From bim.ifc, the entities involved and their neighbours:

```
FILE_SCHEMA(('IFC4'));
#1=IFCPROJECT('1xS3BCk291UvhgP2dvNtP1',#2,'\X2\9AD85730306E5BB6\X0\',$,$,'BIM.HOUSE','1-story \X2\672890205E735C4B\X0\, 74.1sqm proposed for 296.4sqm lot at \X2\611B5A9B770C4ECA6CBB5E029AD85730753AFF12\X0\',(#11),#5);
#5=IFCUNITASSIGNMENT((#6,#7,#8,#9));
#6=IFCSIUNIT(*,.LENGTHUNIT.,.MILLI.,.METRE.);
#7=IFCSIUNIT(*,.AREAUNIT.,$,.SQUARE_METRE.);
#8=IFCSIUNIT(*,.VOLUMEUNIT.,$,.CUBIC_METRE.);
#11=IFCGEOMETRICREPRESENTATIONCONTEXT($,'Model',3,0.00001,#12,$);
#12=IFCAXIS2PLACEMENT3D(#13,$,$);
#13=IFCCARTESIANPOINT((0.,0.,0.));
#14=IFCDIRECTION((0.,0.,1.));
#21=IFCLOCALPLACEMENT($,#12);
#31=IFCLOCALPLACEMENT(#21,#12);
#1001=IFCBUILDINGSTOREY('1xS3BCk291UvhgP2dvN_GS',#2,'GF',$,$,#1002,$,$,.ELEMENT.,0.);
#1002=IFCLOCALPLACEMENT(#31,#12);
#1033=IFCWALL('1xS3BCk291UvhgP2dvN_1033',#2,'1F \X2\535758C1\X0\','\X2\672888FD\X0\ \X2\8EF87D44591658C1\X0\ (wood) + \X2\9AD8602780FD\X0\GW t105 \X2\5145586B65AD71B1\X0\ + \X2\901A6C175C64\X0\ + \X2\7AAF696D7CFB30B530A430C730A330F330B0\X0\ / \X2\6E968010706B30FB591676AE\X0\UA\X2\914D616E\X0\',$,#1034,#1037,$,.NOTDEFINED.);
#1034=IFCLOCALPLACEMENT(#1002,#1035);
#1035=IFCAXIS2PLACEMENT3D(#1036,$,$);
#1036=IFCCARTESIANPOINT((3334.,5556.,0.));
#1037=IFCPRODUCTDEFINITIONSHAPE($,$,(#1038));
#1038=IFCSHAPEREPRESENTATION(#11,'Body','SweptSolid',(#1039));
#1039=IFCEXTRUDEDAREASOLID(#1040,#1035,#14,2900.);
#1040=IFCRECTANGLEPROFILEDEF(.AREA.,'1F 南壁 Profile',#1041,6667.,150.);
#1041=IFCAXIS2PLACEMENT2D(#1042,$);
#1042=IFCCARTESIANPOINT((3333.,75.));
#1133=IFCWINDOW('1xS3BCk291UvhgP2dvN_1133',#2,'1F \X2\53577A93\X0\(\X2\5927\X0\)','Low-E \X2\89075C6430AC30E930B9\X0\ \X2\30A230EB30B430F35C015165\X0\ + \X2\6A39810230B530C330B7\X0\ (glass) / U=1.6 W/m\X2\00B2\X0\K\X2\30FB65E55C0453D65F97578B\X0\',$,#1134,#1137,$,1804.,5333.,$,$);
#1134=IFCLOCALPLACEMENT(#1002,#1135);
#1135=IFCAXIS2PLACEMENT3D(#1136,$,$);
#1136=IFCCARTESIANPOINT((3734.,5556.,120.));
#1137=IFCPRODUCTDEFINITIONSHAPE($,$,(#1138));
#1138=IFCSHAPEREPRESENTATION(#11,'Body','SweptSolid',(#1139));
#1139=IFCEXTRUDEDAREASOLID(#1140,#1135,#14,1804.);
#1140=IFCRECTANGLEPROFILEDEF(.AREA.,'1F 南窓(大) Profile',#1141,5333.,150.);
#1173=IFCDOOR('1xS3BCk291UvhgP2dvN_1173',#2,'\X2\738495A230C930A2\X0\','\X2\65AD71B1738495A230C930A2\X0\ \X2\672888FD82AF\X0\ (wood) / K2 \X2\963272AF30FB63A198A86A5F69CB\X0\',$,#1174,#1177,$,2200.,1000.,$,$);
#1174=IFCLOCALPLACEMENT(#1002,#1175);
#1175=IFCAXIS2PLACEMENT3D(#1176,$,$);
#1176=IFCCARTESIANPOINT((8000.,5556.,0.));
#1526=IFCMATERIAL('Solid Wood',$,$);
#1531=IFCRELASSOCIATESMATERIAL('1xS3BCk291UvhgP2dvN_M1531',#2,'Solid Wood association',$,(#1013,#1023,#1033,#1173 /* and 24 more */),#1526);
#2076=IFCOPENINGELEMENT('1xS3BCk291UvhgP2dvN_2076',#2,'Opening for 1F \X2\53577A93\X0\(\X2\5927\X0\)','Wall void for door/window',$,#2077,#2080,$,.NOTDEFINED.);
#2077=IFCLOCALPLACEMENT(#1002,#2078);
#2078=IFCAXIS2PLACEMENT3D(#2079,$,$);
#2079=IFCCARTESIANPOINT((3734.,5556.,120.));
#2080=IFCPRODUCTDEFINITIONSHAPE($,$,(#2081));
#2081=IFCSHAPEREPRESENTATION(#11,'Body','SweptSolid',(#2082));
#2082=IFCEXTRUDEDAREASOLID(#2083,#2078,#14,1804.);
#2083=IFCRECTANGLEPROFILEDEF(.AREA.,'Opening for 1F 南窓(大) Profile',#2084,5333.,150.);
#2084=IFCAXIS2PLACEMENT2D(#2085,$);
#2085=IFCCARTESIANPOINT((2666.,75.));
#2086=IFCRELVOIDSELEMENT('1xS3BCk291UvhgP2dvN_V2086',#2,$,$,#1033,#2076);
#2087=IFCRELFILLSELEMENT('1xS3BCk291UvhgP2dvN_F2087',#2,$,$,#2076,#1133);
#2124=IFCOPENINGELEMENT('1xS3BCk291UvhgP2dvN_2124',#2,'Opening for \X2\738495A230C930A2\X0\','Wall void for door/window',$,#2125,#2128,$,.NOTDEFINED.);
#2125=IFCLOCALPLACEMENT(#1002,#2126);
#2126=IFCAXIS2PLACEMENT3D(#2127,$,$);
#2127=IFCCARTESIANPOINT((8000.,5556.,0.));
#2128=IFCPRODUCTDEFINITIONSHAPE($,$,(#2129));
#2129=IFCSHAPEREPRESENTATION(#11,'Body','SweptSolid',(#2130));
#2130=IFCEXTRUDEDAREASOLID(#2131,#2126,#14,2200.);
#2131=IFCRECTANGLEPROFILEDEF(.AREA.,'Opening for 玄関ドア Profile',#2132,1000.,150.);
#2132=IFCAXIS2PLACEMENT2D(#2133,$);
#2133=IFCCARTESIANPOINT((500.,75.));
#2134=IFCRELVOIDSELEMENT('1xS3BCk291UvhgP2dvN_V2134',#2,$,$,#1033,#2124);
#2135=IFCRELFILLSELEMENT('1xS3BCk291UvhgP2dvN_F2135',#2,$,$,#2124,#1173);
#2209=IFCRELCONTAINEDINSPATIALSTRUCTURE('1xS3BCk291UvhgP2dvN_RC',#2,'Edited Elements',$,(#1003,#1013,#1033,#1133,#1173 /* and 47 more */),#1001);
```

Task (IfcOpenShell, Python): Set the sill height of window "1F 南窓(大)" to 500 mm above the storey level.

```python
import numpy as np
import ifcopenshell
import ifcopenshell.api.geometry
import ifcopenshell.geom
import ifcopenshell.util.element
import ifcopenshell.util.placement
import ifcopenshell.util.shape
import ifcopenshell.util.unit

model = ifcopenshell.open("bim.ifc")
unit_scale = ifcopenshell.util.unit.calculate_unit_scale(model)

window = model.by_guid("1xS3BCk291UvhgP2dvN_1133")
opening = window.FillsVoids[0].RelatingOpeningElement
storey = ifcopenshell.util.element.get_container(window, ifc_class="IfcBuildingStorey")
level = ifcopenshell.util.placement.get_local_placement(storey.ObjectPlacement)[2, 3]

# The opening's origin need not be at the sill, so measure its lowest point.
shape = ifcopenshell.geom.create_shape(ifcopenshell.geom.settings(), opening)
bottom = ifcopenshell.util.shape.get_shape_bottom_elevation(shape, shape.geometry) / unit_scale
dz = level + 500.0 - bottom

shift = np.array([0.0, 0.0, dz])
# The window is not placed relative to its opening, so move both.
for product in (opening, window):
    matrix = ifcopenshell.util.placement.get_local_placement(product.ObjectPlacement)
    matrix[:3, 3] += shift
    ifcopenshell.api.geometry.edit_object_placement(model, product=product, matrix=matrix, is_si=False)

print(f"moved by {dz * unit_scale:+.3f} m")

model.write("bim_v2.ifc")
```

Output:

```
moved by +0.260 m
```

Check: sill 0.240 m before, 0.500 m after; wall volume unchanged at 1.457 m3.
